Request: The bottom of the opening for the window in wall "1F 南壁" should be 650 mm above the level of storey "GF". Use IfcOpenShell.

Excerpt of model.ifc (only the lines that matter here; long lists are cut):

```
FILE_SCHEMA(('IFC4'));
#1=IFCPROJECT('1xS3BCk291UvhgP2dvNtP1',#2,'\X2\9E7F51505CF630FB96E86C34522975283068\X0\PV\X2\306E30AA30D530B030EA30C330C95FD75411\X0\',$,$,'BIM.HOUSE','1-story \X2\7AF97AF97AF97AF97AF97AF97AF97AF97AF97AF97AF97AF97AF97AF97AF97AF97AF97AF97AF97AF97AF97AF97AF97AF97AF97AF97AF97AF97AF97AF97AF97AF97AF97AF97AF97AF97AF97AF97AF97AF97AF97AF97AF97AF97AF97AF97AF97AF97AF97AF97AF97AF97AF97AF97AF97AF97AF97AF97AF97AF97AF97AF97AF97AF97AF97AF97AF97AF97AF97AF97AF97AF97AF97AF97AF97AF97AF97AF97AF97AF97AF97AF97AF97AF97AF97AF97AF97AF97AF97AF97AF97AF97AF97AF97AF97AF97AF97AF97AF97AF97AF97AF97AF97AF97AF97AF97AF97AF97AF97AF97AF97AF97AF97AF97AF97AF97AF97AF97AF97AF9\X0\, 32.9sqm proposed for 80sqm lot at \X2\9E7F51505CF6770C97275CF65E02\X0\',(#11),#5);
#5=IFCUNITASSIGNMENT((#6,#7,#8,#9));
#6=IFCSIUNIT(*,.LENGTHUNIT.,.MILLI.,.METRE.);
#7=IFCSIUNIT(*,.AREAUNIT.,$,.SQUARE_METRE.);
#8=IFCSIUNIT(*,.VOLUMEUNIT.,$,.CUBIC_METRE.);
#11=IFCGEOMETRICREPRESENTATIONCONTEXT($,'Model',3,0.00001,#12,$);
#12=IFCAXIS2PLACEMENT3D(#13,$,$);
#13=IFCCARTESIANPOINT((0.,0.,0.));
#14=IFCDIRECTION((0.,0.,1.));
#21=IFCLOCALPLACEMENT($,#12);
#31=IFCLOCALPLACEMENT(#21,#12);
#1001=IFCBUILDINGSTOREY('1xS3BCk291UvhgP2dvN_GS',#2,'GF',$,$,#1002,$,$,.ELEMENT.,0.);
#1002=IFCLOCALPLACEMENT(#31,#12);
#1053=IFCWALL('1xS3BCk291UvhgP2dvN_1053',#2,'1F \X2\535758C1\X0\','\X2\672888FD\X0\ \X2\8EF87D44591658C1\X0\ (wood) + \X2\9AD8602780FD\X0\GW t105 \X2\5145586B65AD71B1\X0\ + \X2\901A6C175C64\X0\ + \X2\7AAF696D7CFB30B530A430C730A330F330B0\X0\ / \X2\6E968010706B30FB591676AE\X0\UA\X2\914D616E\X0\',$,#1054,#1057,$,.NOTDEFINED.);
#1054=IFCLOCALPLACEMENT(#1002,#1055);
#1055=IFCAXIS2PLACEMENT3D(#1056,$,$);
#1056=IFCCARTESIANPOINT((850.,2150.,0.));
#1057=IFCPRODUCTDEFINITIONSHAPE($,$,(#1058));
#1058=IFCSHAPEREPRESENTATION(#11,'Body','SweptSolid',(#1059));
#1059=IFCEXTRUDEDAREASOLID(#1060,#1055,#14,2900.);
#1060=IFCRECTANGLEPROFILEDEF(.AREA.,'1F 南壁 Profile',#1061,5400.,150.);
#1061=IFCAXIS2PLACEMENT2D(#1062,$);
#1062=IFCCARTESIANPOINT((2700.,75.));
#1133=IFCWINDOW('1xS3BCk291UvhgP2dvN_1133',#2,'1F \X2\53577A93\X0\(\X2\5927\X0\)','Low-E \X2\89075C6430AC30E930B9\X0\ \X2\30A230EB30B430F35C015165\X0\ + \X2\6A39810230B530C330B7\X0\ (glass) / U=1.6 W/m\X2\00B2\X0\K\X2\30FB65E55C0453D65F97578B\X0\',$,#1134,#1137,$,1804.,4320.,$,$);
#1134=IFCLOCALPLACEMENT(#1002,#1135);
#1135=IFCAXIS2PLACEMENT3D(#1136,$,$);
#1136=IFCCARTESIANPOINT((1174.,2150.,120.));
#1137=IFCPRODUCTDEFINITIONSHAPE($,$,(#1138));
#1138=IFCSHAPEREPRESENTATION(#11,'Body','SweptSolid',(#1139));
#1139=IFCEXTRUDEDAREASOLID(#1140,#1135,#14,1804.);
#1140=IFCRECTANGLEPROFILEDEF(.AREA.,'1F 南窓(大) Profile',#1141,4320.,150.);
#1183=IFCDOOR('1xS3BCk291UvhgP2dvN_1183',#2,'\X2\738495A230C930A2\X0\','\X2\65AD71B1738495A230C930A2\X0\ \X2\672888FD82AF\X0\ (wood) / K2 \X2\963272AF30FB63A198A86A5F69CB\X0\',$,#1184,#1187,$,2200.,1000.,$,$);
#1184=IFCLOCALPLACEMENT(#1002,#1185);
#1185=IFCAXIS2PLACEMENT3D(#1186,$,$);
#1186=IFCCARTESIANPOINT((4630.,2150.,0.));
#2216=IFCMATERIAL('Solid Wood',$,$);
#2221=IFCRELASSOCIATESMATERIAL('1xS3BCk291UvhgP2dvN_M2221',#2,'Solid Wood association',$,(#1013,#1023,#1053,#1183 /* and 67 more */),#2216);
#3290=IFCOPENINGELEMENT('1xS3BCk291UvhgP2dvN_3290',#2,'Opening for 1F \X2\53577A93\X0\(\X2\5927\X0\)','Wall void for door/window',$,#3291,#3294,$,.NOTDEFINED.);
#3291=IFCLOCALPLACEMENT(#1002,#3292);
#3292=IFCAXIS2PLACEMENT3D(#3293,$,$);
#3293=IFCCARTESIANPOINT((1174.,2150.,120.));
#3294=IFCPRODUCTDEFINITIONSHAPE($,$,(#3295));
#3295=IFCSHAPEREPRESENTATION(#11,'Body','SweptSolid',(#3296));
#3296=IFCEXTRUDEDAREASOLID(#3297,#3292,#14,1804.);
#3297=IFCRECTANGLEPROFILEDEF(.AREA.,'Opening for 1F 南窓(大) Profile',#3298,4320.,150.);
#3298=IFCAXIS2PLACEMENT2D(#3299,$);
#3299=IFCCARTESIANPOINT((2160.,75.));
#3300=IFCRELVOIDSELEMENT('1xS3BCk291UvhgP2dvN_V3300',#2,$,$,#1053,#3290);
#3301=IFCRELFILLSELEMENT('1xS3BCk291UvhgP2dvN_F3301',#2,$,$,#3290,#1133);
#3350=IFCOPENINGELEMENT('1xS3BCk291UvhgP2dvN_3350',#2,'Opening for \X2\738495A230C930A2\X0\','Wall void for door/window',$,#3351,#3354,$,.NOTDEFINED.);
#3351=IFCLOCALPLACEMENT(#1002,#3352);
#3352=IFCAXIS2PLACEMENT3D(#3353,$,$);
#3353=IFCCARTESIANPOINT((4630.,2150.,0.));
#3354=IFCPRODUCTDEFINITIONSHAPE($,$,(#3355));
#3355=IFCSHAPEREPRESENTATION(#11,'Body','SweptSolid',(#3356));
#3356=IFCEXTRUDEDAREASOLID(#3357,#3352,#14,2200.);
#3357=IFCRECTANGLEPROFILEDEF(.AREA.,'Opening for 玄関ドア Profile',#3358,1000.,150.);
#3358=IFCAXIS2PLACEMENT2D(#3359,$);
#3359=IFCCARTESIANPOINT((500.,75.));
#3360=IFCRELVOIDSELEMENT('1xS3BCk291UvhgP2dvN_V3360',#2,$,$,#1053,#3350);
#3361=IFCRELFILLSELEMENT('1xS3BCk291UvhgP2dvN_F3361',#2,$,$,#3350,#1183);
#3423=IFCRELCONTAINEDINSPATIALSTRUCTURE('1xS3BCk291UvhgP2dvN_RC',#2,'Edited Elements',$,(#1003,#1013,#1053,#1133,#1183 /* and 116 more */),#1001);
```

```python
import numpy as np
import ifcopenshell
import ifcopenshell.api.geometry
import ifcopenshell.geom
import ifcopenshell.util.element
import ifcopenshell.util.placement
import ifcopenshell.util.shape
import ifcopenshell.util.unit

model = ifcopenshell.open("model.ifc")
unit_scale = ifcopenshell.util.unit.calculate_unit_scale(model)

window = model.by_guid("1xS3BCk291UvhgP2dvN_1133")
opening = window.FillsVoids[0].RelatingOpeningElement
storey = ifcopenshell.util.element.get_container(window, ifc_class="IfcBuildingStorey")
level = ifcopenshell.util.placement.get_local_placement(storey.ObjectPlacement)[2, 3]

# The opening's origin need not be at the sill, so measure its lowest point.
shape = ifcopenshell.geom.create_shape(ifcopenshell.geom.settings(), opening)
bottom = ifcopenshell.util.shape.get_shape_bottom_elevation(shape, shape.geometry) / unit_scale
dz = level + 650.0 - bottom

shift = np.array([0.0, 0.0, dz])
# The window is not placed relative to its opening, so move both.
for product in (opening, window):
    matrix = ifcopenshell.util.placement.get_local_placement(product.ObjectPlacement)
    matrix[:3, 3] += shift
    ifcopenshell.api.geometry.edit_object_placement(model, product=product, matrix=matrix, is_si=False)

print(f"moved by {dz * unit_scale:+.3f} m")

model.write("model_rev.ifc")
```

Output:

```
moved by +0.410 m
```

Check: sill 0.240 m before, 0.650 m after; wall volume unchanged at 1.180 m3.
